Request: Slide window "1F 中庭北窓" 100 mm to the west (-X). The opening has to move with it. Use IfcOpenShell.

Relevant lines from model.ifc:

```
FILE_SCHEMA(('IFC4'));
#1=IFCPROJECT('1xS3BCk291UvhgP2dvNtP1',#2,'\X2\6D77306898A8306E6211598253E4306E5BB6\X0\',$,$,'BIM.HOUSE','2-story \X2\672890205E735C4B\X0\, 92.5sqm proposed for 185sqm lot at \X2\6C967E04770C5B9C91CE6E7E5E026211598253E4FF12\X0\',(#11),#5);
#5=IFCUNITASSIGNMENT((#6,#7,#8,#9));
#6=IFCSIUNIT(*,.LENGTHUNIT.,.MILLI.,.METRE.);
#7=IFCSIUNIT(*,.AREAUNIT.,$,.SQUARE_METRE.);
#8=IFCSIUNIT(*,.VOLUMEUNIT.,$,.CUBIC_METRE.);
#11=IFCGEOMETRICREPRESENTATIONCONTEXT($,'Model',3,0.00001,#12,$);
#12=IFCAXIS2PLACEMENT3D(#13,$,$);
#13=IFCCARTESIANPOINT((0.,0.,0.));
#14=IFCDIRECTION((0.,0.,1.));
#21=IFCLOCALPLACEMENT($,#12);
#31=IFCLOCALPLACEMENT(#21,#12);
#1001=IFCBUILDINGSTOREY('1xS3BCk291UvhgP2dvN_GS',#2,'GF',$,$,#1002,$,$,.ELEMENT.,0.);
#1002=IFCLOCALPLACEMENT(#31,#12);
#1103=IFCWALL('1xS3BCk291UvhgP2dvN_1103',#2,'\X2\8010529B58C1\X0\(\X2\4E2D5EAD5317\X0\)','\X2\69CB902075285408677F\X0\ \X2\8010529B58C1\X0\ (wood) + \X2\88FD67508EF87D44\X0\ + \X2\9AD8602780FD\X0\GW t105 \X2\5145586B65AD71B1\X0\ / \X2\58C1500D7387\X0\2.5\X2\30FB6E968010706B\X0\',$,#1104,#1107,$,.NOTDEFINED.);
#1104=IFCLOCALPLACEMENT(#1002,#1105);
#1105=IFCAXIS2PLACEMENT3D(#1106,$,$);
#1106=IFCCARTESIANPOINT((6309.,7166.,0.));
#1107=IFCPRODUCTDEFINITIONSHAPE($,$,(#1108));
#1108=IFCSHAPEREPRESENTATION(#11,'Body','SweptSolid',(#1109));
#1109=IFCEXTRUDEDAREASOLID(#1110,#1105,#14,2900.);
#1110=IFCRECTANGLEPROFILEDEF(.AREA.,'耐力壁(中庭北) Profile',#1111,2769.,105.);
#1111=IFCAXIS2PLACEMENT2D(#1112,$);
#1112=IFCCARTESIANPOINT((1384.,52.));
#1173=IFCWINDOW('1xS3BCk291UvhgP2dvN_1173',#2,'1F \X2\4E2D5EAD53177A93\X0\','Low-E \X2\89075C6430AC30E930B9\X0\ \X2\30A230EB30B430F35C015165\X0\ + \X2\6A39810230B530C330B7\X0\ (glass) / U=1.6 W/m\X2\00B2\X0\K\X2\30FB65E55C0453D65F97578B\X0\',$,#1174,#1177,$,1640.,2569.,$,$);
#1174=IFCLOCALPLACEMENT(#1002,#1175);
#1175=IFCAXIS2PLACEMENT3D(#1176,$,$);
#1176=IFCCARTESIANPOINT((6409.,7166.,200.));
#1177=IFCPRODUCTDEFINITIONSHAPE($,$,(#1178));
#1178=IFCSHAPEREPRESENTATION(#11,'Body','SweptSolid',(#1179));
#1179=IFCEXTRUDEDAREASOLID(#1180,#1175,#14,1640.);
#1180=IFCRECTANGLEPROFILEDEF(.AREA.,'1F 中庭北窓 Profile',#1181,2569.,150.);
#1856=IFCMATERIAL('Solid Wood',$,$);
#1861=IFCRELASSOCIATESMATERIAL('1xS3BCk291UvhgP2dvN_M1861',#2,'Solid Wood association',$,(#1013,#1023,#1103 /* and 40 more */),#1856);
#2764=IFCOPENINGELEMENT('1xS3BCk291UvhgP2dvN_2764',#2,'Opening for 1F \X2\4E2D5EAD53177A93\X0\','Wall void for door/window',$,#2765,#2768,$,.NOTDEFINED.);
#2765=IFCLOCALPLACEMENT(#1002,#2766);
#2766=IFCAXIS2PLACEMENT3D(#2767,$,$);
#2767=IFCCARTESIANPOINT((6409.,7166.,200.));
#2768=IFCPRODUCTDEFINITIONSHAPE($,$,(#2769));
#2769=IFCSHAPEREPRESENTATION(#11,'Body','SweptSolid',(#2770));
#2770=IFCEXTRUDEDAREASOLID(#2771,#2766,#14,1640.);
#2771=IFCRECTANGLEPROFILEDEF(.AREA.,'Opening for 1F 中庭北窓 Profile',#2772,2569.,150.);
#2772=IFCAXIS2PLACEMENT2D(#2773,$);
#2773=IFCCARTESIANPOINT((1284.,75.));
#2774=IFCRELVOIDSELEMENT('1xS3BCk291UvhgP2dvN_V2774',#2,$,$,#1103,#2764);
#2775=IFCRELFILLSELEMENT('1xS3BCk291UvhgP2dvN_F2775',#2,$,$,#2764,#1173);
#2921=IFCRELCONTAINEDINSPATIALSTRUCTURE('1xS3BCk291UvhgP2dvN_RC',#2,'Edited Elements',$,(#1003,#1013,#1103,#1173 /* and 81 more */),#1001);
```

```python
import ifcopenshell
import ifcopenshell.api.geometry
import ifcopenshell.util.placement

model = ifcopenshell.open("model.ifc")

window = model.by_guid("1xS3BCk291UvhgP2dvN_1173")
opening = window.FillsVoids[0].RelatingOpeningElement
wall = opening.VoidsElements[0].RelatingBuildingElement

wall_matrix = ifcopenshell.util.placement.get_local_placement(wall.ObjectPlacement)
shift = wall_matrix[:3, 0] * -100.0
before = ifcopenshell.util.placement.get_local_placement(window.ObjectPlacement)[:3, 3].copy()

# The window is not placed relative to its opening, so move both.
for product in (opening, window):
    matrix = ifcopenshell.util.placement.get_local_placement(product.ObjectPlacement)
    matrix[:3, 3] += shift
    ifcopenshell.api.geometry.edit_object_placement(model, product=product, matrix=matrix, is_si=False)

after = ifcopenshell.util.placement.get_local_placement(window.ObjectPlacement)[:3, 3]
print("window moved by", (after - before).round(3) + 0.0)

model.write("model_rev.ifc")
```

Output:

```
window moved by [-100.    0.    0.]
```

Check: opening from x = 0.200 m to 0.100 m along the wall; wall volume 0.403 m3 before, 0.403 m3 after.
